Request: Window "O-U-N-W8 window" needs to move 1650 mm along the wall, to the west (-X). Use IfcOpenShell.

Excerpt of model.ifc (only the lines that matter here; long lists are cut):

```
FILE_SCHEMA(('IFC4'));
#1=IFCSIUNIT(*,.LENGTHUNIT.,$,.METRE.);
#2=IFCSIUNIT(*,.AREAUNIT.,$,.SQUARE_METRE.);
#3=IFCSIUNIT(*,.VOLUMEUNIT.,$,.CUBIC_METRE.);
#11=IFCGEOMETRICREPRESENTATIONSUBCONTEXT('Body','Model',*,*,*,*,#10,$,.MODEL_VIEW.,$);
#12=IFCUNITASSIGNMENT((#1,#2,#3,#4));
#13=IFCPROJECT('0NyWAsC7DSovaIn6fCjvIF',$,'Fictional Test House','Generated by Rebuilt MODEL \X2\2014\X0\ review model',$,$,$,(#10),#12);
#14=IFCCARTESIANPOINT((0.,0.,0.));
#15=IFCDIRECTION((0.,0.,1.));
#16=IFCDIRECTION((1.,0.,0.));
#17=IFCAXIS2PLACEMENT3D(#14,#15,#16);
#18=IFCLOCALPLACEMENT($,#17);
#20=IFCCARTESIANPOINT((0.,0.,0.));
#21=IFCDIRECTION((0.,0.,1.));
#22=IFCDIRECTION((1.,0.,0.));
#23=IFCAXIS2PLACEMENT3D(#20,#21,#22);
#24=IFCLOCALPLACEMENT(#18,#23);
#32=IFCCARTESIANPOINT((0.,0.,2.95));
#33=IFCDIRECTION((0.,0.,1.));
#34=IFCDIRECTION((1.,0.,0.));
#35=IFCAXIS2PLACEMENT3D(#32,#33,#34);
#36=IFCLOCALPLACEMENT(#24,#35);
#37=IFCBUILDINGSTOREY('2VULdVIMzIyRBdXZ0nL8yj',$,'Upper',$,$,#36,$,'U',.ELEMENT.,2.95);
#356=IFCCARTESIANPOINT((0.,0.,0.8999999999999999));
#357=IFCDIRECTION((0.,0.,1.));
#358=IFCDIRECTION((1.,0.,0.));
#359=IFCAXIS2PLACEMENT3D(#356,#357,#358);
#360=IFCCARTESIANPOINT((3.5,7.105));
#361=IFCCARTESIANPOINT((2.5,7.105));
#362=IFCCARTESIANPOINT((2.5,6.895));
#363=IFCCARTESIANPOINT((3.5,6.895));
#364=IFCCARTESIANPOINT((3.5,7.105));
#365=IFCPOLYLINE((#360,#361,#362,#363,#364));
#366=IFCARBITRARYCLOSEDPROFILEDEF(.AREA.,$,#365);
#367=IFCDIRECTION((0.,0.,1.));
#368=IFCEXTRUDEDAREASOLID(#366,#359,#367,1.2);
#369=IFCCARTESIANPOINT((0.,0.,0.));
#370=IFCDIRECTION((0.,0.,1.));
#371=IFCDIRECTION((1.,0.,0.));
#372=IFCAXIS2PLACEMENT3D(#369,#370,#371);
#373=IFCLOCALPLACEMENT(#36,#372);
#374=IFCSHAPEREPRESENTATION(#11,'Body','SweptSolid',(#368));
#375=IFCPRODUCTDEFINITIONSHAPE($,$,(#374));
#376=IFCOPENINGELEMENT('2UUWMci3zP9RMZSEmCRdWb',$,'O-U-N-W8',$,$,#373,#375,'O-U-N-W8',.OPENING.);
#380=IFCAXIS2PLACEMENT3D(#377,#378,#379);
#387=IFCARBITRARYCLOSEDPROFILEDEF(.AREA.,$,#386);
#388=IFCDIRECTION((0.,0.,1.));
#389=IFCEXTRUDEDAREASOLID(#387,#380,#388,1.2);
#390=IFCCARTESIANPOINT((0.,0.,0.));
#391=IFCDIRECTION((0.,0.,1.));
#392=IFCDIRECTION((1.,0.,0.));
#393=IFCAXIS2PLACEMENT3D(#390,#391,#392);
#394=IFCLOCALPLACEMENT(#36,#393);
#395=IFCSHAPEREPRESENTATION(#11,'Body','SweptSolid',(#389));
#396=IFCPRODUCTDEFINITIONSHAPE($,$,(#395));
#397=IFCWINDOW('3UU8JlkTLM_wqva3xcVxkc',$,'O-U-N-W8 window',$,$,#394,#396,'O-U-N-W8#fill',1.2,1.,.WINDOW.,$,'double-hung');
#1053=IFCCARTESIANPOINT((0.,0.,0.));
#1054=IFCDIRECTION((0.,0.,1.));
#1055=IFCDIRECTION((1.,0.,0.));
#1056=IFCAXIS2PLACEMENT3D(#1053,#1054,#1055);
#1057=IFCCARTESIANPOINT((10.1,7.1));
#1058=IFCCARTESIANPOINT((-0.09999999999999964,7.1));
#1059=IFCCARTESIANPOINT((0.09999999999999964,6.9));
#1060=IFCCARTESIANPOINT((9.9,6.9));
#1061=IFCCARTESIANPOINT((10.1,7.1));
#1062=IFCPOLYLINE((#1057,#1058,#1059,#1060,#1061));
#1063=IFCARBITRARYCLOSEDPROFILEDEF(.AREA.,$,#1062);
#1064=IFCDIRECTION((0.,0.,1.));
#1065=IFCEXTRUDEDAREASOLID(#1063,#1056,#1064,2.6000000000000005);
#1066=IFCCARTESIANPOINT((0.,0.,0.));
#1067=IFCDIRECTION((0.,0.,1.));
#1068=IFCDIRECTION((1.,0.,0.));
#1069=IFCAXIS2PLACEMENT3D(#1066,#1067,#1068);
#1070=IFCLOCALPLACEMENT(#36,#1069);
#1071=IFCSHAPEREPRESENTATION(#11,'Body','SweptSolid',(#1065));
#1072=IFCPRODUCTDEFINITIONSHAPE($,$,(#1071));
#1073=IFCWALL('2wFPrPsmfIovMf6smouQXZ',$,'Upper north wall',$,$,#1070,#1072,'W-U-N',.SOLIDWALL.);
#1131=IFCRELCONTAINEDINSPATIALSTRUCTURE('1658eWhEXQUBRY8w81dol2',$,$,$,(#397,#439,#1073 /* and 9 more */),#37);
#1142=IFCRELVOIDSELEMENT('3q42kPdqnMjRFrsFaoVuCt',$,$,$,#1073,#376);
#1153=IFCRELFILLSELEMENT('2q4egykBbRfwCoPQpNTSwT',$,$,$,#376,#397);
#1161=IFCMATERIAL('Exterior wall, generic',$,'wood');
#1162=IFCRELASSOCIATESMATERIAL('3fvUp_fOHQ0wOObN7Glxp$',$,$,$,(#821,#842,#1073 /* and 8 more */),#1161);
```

```python
import ifcopenshell
import ifcopenshell.api.geometry
import ifcopenshell.util.placement
import ifcopenshell.util.unit

model = ifcopenshell.open("model.ifc")
unit_scale = ifcopenshell.util.unit.calculate_unit_scale(model)

window = model.by_guid("3UU8JlkTLM_wqva3xcVxkc")
opening = window.FillsVoids[0].RelatingOpeningElement
wall = opening.VoidsElements[0].RelatingBuildingElement

wall_matrix = ifcopenshell.util.placement.get_local_placement(wall.ObjectPlacement)
shift = wall_matrix[:3, 0] * -1.65 / unit_scale
before = ifcopenshell.util.placement.get_local_placement(window.ObjectPlacement)[:3, 3].copy()

# The window is not placed relative to its opening, so move both.
for product in (opening, window):
    matrix = ifcopenshell.util.placement.get_local_placement(product.ObjectPlacement)
    matrix[:3, 3] += shift
    ifcopenshell.api.geometry.edit_object_placement(model, product=product, matrix=matrix, is_si=False)

after = ifcopenshell.util.placement.get_local_placement(window.ObjectPlacement)[:3, 3]
print("window moved by", (after - before).round(3) + 0.0)

model.write("model_edited.ifc")
```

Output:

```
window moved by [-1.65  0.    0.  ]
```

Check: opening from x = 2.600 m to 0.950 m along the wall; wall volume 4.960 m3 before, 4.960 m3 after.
